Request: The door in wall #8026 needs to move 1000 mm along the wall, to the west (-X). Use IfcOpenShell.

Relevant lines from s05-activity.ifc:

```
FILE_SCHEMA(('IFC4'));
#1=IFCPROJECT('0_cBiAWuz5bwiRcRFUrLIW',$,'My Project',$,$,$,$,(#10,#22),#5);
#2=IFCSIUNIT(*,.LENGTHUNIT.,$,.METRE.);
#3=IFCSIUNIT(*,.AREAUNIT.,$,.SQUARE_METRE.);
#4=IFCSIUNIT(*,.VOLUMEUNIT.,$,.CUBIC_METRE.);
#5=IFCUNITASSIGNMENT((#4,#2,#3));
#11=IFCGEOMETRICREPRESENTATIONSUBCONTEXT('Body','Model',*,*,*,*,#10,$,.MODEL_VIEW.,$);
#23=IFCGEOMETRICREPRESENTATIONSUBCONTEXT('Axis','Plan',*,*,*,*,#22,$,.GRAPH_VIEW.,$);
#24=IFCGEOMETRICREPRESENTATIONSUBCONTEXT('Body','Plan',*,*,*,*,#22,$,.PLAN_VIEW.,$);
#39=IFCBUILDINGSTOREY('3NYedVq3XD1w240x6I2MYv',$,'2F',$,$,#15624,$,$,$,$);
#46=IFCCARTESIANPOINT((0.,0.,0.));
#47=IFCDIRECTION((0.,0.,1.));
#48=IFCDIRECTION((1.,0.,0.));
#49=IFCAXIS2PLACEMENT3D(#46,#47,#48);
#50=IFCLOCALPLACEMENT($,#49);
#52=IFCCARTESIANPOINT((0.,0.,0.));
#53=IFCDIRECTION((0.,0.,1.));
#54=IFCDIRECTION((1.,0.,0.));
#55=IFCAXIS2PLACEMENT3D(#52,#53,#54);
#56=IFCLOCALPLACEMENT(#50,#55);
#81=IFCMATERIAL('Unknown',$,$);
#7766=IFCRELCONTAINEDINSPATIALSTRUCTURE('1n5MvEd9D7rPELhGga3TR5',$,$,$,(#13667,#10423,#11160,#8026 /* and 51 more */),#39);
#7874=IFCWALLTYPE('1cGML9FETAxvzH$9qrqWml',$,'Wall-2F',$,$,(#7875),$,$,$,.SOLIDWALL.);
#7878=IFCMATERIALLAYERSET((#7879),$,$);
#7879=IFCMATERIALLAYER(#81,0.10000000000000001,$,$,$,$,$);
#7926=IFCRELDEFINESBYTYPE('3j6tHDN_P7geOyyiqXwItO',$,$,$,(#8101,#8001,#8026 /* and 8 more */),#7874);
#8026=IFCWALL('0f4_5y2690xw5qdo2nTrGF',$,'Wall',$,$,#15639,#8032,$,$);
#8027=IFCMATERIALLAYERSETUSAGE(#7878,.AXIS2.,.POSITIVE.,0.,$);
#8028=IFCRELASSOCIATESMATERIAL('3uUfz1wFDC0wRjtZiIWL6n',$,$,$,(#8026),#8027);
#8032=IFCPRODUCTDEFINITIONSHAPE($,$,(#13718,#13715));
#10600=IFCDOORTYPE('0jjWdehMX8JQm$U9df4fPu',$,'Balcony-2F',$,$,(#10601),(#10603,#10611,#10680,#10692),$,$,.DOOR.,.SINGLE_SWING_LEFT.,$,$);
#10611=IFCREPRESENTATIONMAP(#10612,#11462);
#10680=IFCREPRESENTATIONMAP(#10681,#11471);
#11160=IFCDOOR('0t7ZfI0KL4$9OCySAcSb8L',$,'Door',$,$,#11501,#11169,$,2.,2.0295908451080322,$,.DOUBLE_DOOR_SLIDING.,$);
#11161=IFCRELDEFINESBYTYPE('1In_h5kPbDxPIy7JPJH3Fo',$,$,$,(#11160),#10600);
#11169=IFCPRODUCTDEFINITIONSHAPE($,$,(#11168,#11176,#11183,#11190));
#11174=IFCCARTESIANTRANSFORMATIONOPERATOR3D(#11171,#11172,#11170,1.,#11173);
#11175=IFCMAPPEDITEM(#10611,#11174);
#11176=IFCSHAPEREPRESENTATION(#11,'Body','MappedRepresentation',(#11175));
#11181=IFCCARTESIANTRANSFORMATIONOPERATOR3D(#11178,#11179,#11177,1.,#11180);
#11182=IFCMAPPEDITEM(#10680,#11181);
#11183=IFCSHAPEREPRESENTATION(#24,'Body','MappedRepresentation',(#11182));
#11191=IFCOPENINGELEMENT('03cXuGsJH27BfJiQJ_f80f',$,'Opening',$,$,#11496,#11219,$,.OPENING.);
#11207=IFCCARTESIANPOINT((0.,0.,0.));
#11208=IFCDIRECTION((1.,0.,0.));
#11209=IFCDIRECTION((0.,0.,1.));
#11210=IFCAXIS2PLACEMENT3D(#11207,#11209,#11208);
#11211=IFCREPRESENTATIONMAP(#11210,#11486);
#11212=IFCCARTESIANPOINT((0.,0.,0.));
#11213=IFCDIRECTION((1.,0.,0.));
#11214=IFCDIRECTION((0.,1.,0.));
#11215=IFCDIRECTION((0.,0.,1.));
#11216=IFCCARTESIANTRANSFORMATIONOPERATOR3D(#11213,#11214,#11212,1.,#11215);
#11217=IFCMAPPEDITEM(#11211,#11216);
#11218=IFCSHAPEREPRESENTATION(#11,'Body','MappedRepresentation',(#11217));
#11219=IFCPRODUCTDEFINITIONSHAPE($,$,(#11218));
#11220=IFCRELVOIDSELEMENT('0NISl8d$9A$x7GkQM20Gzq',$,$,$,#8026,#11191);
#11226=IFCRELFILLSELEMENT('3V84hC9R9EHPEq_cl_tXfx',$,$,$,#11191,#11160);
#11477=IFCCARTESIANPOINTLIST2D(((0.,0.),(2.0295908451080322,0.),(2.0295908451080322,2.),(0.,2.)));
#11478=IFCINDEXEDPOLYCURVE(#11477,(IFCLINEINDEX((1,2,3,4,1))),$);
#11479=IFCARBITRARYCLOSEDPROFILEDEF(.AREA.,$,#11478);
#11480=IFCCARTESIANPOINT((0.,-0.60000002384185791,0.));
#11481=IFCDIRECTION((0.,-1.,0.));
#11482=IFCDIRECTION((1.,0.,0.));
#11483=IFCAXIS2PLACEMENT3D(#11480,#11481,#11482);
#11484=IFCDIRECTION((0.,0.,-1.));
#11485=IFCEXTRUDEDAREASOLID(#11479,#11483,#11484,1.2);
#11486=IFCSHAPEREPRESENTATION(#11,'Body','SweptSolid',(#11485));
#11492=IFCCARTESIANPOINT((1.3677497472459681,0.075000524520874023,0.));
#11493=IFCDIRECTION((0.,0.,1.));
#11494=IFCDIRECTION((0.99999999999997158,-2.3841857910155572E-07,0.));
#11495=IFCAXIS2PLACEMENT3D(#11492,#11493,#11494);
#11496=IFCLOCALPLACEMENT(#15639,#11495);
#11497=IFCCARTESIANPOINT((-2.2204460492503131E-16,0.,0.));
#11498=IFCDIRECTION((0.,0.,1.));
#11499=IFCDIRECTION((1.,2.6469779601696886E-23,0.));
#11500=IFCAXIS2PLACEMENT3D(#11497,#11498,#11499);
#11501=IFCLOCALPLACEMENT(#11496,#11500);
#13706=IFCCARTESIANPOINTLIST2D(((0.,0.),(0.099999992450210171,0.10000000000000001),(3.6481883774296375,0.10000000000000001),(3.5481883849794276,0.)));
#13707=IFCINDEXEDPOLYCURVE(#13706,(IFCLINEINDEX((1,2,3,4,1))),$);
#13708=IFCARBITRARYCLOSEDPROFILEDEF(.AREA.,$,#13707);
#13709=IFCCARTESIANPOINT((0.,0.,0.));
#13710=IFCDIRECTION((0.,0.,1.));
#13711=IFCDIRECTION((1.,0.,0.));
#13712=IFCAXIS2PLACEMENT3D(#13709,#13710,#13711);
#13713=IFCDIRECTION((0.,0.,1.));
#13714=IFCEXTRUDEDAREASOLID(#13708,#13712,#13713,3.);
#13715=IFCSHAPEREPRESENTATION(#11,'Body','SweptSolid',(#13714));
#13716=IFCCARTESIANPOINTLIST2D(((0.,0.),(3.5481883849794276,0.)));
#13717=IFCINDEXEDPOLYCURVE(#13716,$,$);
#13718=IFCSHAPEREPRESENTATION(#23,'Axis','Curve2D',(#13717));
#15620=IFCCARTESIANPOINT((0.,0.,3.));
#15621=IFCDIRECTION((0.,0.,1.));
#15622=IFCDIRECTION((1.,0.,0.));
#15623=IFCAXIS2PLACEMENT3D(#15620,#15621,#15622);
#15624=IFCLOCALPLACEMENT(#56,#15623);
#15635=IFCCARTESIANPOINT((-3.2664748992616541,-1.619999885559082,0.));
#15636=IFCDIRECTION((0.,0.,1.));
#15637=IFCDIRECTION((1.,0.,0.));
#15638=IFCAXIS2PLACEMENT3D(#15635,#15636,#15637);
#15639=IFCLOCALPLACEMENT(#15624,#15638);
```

```python
import ifcopenshell
import ifcopenshell.api.geometry
import ifcopenshell.util.placement
import ifcopenshell.util.unit

model = ifcopenshell.open("s05-activity.ifc")
unit_scale = ifcopenshell.util.unit.calculate_unit_scale(model)

door = model.by_guid("0t7ZfI0KL4$9OCySAcSb8L")
opening = door.FillsVoids[0].RelatingOpeningElement
wall = opening.VoidsElements[0].RelatingBuildingElement

wall_matrix = ifcopenshell.util.placement.get_local_placement(wall.ObjectPlacement)
shift = wall_matrix[:3, 0] * -1 / unit_scale
before = ifcopenshell.util.placement.get_local_placement(door.ObjectPlacement)[:3, 3].copy()

# The door is placed relative to its opening, so it follows when the opening moves.
matrix = ifcopenshell.util.placement.get_local_placement(opening.ObjectPlacement)
matrix[:3, 3] += shift
ifcopenshell.api.geometry.edit_object_placement(
    model, product=opening, matrix=matrix, is_si=False, should_transform_children=True
)

after = ifcopenshell.util.placement.get_local_placement(door.ObjectPlacement)[:3, 3]
print("door moved by", (after - before).round(3) + 0.0)

model.write("s05-activity_rev.ifc")
```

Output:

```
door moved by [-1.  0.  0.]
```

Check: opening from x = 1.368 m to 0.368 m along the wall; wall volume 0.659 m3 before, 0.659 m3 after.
